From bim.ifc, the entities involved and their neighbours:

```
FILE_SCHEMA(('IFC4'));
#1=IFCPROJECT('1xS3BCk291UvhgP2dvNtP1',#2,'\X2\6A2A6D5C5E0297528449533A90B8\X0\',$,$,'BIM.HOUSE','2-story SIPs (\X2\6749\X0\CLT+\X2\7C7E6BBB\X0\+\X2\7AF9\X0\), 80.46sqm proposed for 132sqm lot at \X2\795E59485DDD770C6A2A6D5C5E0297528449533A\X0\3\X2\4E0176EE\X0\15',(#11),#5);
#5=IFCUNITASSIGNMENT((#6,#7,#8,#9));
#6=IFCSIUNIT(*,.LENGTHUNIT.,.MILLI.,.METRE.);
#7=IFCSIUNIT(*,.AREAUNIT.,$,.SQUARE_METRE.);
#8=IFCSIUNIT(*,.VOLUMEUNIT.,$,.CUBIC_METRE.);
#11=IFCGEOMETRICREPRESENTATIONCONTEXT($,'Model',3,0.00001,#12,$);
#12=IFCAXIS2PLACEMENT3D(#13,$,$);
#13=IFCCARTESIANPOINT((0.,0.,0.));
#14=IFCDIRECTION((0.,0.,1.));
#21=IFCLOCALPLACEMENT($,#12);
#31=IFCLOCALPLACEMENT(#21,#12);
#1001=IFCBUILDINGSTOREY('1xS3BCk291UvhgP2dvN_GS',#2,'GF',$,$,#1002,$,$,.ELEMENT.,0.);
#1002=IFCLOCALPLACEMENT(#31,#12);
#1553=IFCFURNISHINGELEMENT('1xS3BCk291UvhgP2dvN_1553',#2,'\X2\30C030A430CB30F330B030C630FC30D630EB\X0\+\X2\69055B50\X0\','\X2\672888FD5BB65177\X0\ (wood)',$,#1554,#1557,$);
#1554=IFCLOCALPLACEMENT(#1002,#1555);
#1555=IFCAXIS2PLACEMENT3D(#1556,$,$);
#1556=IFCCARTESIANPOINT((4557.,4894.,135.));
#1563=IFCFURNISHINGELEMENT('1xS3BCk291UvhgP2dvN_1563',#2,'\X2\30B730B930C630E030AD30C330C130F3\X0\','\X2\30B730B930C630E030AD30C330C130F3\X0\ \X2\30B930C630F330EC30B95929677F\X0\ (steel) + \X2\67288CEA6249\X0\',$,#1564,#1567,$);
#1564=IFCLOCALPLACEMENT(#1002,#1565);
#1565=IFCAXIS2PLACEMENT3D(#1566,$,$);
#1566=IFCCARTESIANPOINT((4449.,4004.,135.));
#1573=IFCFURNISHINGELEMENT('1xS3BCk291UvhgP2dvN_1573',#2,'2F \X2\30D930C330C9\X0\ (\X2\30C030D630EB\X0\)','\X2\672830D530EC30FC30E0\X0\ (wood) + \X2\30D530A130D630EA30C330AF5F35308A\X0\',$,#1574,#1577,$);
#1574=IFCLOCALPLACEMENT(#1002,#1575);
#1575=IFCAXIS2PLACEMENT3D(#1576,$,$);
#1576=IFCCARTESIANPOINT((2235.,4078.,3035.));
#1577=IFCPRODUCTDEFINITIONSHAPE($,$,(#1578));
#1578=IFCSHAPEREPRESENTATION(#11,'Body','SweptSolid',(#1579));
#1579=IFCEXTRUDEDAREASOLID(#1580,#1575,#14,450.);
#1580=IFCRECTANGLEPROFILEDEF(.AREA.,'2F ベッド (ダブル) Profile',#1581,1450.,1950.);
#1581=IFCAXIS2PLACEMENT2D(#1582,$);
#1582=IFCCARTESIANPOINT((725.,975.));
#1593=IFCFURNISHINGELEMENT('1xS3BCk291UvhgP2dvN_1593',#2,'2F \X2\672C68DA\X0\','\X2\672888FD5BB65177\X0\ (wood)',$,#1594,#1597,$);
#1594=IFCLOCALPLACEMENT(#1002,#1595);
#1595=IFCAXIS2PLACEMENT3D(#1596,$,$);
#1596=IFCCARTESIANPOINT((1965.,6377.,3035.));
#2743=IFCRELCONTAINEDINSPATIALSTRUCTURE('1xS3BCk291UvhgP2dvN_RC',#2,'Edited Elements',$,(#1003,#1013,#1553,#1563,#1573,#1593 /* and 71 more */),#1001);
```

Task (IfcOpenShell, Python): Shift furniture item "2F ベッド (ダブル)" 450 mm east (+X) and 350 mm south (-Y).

```python
import ifcopenshell
import ifcopenshell.api.geometry
import ifcopenshell.util.placement
import ifcopenshell.util.unit

model = ifcopenshell.open("bim.ifc")
unit_scale = ifcopenshell.util.unit.calculate_unit_scale(model)

item = model.by_guid("1xS3BCk291UvhgP2dvN_1573")
matrix = ifcopenshell.util.placement.get_local_placement(item.ObjectPlacement)
matrix[0, 3] += 0.45 / unit_scale
matrix[1, 3] -= 0.35 / unit_scale
ifcopenshell.api.geometry.edit_object_placement(model, product=item, matrix=matrix, is_si=False)

print(ifcopenshell.util.placement.get_local_placement(item.ObjectPlacement).round(3) + 0.0)

model.write("bim_updated.ifc")
```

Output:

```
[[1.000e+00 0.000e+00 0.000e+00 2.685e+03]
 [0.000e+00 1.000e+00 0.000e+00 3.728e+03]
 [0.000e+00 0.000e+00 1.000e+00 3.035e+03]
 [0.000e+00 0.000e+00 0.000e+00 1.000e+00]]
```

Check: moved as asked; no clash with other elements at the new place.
